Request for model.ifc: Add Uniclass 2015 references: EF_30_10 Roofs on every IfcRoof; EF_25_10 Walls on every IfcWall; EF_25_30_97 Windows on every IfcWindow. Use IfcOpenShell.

First a look at what the model holds.

```python
import ifcopenshell

model = ifcopenshell.open("model.ifc")
print(model.schema)
print("classifications:", [c.Name for c in model.by_type("IfcClassification")])
for ifc_class in ("IfcDoor", "IfcRoof", "IfcStair", "IfcWall", "IfcWindow"):
    print(ifc_class, len(model.by_type(ifc_class)))
```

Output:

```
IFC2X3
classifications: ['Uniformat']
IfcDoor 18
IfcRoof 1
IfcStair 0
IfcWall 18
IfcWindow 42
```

```python
import ifcopenshell
import ifcopenshell.api.classification

model = ifcopenshell.open("model.ifc")

# IFC2X3 requires Source and Edition and has no link from the project to the system.
system = model.create_entity("IfcClassification", Source="NBS", Edition="2015", Name="Uniclass 2015")

codes = {
    "IfcRoof": ("EF_30_10", "Roofs"),
    "IfcWall": ("EF_25_10", "Walls"),
    "IfcWindow": ("EF_25_30_97", "Windows"),
}
for ifc_class, (code, name) in codes.items():
    products = model.by_type(ifc_class)
    ifcopenshell.api.classification.add_reference(
        model, products=products, classification=system, identification=code, name=name
    )
    print(code, len(products))

model.write("model_updated.ifc")
```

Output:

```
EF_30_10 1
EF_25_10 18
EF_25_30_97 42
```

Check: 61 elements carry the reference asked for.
